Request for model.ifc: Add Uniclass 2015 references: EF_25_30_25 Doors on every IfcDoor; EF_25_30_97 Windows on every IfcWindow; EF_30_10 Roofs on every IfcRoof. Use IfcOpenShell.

First a look at what the model holds.

```python
import ifcopenshell

model = ifcopenshell.open("model.ifc")
print(model.schema)
print("classifications:", [c.Name for c in model.by_type("IfcClassification")])
for ifc_class in ("IfcDoor", "IfcRoof", "IfcStair", "IfcWall", "IfcWindow"):
    print(ifc_class, len(model.by_type(ifc_class)))
```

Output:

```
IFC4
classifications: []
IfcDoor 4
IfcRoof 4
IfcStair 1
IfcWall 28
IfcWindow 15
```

```python
import ifcopenshell
import ifcopenshell.api.classification

model = ifcopenshell.open("model.ifc")

system = ifcopenshell.api.classification.add_classification(model, classification="Uniclass 2015")

codes = {
    "IfcDoor": ("EF_25_30_25", "Doors"),
    "IfcWindow": ("EF_25_30_97", "Windows"),
    "IfcRoof": ("EF_30_10", "Roofs"),
}
for ifc_class, (code, name) in codes.items():
    products = model.by_type(ifc_class)
    ifcopenshell.api.classification.add_reference(
        model, products=products, classification=system, identification=code, name=name
    )
    print(code, len(products))

model.write("model_v2.ifc")
```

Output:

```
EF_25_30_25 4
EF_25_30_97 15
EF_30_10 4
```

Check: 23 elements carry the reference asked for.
